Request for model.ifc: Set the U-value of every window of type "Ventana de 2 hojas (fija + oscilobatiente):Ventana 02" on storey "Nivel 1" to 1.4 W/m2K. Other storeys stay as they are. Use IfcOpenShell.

First a look at what the model holds.

```python
import ifcopenshell
import ifcopenshell.util.element

model = ifcopenshell.open("model.ifc")
print(model.schema)
storey = next(s for s in model.by_type("IfcBuildingStorey") if s.Name == "Nivel 1")
windows = [e for e in ifcopenshell.util.element.get_decomposition(storey) if e.is_a("IfcWindow")]
seen = {}
for e in windows:
    element_type = ifcopenshell.util.element.get_type(e)
    key = (element_type.Name if element_type != e and element_type else None, ifcopenshell.util.element.get_pset(e, "Pset_WindowCommon", "ThermalTransmittance"))
    seen[key] = seen.get(key, 0) + 1
for (name, value), count in sorted(seen.items(), key=str):
    print(count, "x", name, "|", value)
```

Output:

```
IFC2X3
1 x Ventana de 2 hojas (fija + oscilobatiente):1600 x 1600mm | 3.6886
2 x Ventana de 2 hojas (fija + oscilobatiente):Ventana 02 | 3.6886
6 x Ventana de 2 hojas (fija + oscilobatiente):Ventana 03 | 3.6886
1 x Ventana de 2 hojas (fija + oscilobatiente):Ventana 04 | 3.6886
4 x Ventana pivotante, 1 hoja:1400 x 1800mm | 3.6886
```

```python
import ifcopenshell
import ifcopenshell.api.pset
import ifcopenshell.util.element

model = ifcopenshell.open("model.ifc")

storey = next(s for s in model.by_type("IfcBuildingStorey") if s.Name == "Nivel 1")
windows = [e for e in ifcopenshell.util.element.get_decomposition(storey) if e.is_a("IfcWindow")]

count = 0
for e in windows:
    element_type = ifcopenshell.util.element.get_type(e)
    if element_type in (None, e) or element_type.Name != "Ventana de 2 hojas (fija + oscilobatiente):Ventana 02":
        continue
    # add_pset returns the element's existing set when there is one.
    pset = ifcopenshell.api.pset.add_pset(model, product=e, name="Pset_WindowCommon")
    ifcopenshell.api.pset.edit_pset(model, pset=pset, properties={"ThermalTransmittance": 1.4})
    count += 1

print(count, "windows updated")

model.write("model_rev.ifc")
```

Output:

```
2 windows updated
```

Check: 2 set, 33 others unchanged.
